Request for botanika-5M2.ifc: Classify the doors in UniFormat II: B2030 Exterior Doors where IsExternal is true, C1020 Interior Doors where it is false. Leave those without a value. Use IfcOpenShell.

First a look at what the model holds.

```python
import ifcopenshell
import ifcopenshell.util.element

model = ifcopenshell.open("botanika-5M2.ifc")
print(model.schema)
print("classifications:", [c.Name for c in model.by_type("IfcClassification")])
values = [ifcopenshell.util.element.get_pset(e, "Pset_DoorCommon", "IsExternal") for e in model.by_type("IfcDoor")]
for value in (True, False, None):
    print("IsExternal", value, values.count(value))
```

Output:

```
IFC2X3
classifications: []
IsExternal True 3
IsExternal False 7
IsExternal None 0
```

```python
import ifcopenshell
import ifcopenshell.api.classification
import ifcopenshell.util.element

model = ifcopenshell.open("botanika-5M2.ifc")

# IFC2X3 requires Source and Edition and has no link from the project to the system.
system = model.create_entity("IfcClassification", Source="ASTM", Edition="E1557", Name="UniFormat II")

doors = model.by_type("IfcDoor")
external = {e: ifcopenshell.util.element.get_pset(e, "Pset_DoorCommon", "IsExternal") for e in doors}
for flag, code, name in ((True, "B2030", "Exterior Doors"), (False, "C1020", "Interior Doors")):
    products = [e for e in doors if external[e] is flag]
    ifcopenshell.api.classification.add_reference(
        model, products=products, classification=system, identification=code, name=name
    )
    print(code, len(products))

model.write("botanika-5M2_v2.ifc")
```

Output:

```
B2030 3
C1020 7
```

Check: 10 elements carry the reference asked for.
